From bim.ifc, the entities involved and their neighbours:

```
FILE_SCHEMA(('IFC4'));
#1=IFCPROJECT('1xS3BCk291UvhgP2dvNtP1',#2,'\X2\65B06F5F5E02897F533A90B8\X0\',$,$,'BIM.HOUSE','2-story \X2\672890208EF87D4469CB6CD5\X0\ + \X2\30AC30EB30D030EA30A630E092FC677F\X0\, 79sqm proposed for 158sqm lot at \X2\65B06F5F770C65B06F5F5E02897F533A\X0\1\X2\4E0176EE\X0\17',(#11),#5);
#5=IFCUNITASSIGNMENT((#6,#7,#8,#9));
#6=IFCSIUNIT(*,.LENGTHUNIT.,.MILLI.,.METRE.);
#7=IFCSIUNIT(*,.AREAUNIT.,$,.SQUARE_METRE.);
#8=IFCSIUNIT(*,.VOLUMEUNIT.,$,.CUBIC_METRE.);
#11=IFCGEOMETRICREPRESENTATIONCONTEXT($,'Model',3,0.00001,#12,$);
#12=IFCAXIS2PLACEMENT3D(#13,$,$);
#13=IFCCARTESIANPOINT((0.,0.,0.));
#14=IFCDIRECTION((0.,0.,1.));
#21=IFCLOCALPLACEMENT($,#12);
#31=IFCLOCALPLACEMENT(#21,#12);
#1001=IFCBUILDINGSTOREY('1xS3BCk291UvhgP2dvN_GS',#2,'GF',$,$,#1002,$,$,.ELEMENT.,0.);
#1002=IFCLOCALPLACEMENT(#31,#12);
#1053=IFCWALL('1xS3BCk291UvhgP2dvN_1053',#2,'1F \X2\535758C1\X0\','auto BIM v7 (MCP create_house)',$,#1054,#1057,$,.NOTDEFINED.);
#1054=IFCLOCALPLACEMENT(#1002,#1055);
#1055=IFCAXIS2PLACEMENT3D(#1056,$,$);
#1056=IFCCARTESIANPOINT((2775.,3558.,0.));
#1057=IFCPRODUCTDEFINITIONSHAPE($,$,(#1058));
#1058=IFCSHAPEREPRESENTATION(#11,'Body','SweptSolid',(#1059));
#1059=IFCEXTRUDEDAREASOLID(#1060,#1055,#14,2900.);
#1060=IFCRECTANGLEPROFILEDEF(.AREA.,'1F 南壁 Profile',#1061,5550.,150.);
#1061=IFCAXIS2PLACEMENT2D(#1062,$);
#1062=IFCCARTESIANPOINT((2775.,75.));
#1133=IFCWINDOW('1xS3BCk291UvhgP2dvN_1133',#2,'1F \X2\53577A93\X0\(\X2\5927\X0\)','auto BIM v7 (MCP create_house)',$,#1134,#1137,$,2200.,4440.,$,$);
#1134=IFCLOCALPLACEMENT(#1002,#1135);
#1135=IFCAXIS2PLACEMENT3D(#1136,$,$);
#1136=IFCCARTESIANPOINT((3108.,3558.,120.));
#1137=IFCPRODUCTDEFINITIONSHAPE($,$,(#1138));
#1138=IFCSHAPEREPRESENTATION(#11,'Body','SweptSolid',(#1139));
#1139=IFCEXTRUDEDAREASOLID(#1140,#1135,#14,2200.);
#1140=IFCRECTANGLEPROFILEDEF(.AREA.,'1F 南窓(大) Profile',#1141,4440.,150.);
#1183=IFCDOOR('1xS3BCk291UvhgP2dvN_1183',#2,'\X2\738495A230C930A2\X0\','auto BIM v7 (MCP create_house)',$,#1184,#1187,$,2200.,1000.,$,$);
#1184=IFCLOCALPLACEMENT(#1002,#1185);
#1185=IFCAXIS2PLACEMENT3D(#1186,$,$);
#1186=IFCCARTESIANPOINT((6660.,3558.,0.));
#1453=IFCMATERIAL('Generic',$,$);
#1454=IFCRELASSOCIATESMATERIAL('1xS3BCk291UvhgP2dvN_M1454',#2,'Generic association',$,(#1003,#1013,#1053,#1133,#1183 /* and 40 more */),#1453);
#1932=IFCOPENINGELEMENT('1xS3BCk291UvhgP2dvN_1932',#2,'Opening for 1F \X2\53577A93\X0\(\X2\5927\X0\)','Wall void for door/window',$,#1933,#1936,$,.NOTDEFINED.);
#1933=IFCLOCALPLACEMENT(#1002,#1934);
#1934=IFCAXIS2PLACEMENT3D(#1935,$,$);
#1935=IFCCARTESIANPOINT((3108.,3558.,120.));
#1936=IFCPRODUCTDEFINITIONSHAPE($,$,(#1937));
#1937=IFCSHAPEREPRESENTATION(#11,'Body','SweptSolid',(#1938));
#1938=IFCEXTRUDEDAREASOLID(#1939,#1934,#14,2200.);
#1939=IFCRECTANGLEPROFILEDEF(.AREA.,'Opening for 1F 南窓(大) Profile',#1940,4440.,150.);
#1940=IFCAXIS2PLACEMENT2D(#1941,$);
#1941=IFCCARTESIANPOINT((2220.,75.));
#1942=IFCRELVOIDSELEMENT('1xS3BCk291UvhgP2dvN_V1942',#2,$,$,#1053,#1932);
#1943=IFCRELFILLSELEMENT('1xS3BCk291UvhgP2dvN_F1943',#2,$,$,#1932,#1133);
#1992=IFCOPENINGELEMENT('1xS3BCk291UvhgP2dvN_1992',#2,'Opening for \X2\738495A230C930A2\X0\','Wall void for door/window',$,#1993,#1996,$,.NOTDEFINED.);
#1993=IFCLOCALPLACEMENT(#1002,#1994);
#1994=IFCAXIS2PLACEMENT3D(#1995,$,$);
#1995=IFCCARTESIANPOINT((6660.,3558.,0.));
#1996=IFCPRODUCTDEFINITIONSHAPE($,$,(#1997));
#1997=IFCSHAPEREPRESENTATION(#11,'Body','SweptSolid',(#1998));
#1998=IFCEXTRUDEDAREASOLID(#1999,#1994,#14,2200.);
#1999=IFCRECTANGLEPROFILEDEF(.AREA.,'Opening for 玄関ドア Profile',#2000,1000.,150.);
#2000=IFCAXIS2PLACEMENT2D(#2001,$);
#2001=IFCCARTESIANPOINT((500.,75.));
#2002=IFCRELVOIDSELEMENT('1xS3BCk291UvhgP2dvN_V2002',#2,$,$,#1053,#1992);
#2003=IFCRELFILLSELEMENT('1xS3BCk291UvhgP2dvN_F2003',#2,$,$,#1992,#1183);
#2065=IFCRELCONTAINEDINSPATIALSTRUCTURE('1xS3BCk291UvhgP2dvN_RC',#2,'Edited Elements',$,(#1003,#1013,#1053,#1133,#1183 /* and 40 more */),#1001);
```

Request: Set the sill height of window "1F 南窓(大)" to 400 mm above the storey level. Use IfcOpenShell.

```python
import numpy as np
import ifcopenshell
import ifcopenshell.api.geometry
import ifcopenshell.geom
import ifcopenshell.util.element
import ifcopenshell.util.placement
import ifcopenshell.util.shape
import ifcopenshell.util.unit

model = ifcopenshell.open("bim.ifc")
unit_scale = ifcopenshell.util.unit.calculate_unit_scale(model)

window = model.by_id(1133)
opening = window.FillsVoids[0].RelatingOpeningElement
storey = ifcopenshell.util.element.get_container(window, ifc_class="IfcBuildingStorey")
level = ifcopenshell.util.placement.get_local_placement(storey.ObjectPlacement)[2, 3]

# The opening's origin need not be at the sill, so measure its lowest point.
shape = ifcopenshell.geom.create_shape(ifcopenshell.geom.settings(), opening)
bottom = ifcopenshell.util.shape.get_shape_bottom_elevation(shape, shape.geometry) / unit_scale
dz = level + 0.4 / unit_scale - bottom

shift = np.array([0.0, 0.0, dz])
# The window is not placed relative to its opening, so move both.
for product in (opening, window):
    matrix = ifcopenshell.util.placement.get_local_placement(product.ObjectPlacement)
    matrix[:3, 3] += shift
    ifcopenshell.api.geometry.edit_object_placement(model, product=product, matrix=matrix, is_si=False)

print(f"moved by {dz * unit_scale:+.3f} m")

model.write("bim_updated.ifc")
```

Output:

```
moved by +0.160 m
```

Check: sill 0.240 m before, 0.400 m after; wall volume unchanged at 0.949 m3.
